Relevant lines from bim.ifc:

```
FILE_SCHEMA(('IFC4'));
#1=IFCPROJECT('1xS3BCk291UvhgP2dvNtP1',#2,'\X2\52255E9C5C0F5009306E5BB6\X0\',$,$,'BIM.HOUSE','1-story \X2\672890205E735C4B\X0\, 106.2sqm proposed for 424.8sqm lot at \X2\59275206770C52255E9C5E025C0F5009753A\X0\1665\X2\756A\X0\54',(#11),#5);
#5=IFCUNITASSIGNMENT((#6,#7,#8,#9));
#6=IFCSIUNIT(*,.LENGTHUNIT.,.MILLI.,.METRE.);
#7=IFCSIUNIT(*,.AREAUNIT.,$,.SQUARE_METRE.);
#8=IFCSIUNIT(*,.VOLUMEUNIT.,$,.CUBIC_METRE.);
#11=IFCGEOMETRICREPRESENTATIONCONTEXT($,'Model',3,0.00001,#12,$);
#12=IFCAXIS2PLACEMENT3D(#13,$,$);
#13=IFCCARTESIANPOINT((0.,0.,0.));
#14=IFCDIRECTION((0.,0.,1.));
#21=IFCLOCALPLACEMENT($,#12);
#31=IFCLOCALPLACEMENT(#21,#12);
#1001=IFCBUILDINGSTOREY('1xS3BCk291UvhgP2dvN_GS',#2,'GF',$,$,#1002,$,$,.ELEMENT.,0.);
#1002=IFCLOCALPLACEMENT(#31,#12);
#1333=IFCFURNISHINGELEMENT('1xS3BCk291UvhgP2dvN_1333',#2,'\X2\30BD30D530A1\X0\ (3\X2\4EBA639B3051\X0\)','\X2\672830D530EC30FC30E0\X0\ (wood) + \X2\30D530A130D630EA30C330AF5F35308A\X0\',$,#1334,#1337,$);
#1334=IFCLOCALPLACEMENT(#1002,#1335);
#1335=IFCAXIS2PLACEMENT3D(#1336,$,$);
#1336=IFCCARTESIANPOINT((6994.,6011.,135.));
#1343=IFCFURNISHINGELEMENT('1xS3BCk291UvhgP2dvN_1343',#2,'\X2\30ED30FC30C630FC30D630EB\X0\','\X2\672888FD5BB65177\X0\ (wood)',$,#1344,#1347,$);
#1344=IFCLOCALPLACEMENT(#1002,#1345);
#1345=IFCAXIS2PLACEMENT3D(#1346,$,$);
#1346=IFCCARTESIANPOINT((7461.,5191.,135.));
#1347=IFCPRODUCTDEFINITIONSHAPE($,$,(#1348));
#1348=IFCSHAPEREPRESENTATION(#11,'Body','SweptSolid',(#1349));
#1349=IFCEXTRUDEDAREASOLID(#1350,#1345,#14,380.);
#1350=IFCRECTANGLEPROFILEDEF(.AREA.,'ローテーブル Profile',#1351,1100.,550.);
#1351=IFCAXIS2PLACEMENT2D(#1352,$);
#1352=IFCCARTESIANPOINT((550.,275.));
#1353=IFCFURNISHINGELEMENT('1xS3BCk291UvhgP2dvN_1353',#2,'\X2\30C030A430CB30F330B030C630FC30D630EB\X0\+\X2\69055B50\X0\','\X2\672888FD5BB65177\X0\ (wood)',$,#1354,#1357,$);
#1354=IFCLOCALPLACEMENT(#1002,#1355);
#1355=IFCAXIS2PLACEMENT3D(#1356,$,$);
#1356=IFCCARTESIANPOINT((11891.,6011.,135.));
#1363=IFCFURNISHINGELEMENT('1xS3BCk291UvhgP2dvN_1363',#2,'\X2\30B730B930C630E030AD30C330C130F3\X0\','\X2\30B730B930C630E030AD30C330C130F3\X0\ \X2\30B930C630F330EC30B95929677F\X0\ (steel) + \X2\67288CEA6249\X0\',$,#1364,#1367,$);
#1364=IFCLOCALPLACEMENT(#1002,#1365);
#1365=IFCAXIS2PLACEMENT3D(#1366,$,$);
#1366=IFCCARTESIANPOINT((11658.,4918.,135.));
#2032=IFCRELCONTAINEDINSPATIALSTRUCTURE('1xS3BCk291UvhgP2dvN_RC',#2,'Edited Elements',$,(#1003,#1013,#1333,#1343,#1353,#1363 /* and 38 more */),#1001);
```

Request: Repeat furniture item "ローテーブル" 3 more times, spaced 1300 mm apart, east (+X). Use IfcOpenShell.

```python
import numpy as np
import ifcopenshell
import ifcopenshell.api.geometry
import ifcopenshell.api.root
import ifcopenshell.util.element
import ifcopenshell.util.placement
import ifcopenshell.util.unit

model = ifcopenshell.open("bim.ifc")
unit_scale = ifcopenshell.util.unit.calculate_unit_scale(model)


def reuse_history(source, copy):
    """copy_class also copies each property set's owner history, people and application; keep the originals."""
    for rel in copy.IsDefinedBy:
        if rel.is_a("IfcRelDefinesByProperties") and (history := rel.RelatingPropertyDefinition.OwnerHistory):
            rel.RelatingPropertyDefinition.OwnerHistory = source.OwnerHistory
            ifcopenshell.util.element.remove_deep2(model, history)


source = model.by_guid("1xS3BCk291UvhgP2dvN_1343")
base = ifcopenshell.util.placement.get_local_placement(source.ObjectPlacement)
step = np.array([1.0, 0.0, 0.0]) * 1.3 / unit_scale

for i in range(1, 4):
    copy = ifcopenshell.api.root.copy_class(model, product=source)
    copy.Representation = ifcopenshell.util.element.copy_deep(
        model, source.Representation, exclude=["IfcGeometricRepresentationContext", "IfcRepresentationMap"]
    )
    reuse_history(source, copy)
    matrix = base.copy()
    matrix[:3, 3] += i * step
    print("added at", matrix[:3, 3].round(3) + 0.0)
    ifcopenshell.api.geometry.edit_object_placement(model, product=copy, matrix=matrix, is_si=False)

model.write("bim_v2.ifc")
```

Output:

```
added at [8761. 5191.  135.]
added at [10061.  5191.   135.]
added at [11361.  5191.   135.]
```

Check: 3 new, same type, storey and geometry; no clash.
